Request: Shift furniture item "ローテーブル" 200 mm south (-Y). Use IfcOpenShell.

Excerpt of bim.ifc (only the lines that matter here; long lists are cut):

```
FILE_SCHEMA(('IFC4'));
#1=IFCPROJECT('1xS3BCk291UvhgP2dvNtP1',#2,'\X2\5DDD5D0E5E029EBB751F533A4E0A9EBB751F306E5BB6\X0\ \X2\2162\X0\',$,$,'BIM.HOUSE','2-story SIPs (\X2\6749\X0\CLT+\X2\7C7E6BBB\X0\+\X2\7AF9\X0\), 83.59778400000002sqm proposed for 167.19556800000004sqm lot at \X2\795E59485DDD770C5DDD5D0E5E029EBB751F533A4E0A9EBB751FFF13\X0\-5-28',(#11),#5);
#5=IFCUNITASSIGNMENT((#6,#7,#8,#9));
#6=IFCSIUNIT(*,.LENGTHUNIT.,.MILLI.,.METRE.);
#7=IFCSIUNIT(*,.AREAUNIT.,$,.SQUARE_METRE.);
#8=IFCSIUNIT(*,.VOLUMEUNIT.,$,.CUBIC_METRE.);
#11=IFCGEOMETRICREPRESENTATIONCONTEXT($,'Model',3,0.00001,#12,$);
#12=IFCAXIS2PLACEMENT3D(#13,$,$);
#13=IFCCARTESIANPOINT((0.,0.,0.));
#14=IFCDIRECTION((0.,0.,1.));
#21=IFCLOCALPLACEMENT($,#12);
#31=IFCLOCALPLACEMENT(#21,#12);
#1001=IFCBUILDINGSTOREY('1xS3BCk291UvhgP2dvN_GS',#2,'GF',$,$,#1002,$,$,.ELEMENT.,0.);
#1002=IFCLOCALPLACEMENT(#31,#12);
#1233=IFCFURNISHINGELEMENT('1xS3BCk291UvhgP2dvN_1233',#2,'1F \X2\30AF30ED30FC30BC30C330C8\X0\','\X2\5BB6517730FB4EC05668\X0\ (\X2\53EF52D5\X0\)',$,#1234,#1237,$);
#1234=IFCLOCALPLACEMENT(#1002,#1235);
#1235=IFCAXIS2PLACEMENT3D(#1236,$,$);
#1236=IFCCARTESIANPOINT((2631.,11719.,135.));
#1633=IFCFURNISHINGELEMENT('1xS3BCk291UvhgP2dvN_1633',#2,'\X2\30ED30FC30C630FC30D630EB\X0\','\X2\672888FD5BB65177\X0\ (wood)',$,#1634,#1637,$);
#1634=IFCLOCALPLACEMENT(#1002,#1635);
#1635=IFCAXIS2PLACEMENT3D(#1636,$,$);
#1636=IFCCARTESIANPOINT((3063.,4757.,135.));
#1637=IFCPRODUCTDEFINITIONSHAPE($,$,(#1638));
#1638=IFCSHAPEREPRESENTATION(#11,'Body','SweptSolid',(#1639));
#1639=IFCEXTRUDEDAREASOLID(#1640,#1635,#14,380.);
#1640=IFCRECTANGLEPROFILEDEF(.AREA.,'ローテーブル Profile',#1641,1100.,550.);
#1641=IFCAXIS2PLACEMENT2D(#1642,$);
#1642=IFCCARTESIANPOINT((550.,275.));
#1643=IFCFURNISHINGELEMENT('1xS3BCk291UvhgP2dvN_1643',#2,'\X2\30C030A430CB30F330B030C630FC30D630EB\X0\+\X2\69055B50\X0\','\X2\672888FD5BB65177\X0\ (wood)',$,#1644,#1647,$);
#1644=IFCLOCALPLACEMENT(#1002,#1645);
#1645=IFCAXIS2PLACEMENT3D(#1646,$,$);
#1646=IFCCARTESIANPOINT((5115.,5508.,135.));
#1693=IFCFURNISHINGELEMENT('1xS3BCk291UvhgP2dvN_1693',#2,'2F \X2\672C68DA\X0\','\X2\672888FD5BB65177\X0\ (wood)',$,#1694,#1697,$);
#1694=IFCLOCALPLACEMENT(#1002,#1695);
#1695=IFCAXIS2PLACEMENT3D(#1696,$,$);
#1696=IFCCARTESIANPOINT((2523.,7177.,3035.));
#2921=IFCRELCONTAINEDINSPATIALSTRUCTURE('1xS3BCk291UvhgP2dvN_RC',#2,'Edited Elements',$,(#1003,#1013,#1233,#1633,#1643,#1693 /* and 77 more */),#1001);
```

```python
import ifcopenshell
import ifcopenshell.api.geometry
import ifcopenshell.util.placement
import ifcopenshell.util.unit

model = ifcopenshell.open("bim.ifc")
unit_scale = ifcopenshell.util.unit.calculate_unit_scale(model)

item = model.by_guid("1xS3BCk291UvhgP2dvN_1633")
matrix = ifcopenshell.util.placement.get_local_placement(item.ObjectPlacement)
matrix[1, 3] -= 0.2 / unit_scale
ifcopenshell.api.geometry.edit_object_placement(model, product=item, matrix=matrix, is_si=False)

print(ifcopenshell.util.placement.get_local_placement(item.ObjectPlacement).round(3) + 0.0)

model.write("bim_v2.ifc")
```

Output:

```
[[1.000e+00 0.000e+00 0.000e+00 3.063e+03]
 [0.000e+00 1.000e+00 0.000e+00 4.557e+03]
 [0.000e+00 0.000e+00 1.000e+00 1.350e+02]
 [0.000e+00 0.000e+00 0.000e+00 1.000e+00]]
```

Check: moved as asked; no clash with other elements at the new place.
